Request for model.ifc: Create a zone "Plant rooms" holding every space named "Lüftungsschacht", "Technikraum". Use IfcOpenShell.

First a look at what the model holds.

```python
import ifcopenshell

model = ifcopenshell.open("model.ifc")
print(model.schema)
seen = {}
for space in model.by_type("IfcSpace"):
    seen[space.LongName] = seen.get(space.LongName, 0) + 1
for name, count in sorted(seen.items(), key=str):
    print(count, "x", name)
print("zones:", [z.Name for z in model.by_type("IfcZone")][:20])
```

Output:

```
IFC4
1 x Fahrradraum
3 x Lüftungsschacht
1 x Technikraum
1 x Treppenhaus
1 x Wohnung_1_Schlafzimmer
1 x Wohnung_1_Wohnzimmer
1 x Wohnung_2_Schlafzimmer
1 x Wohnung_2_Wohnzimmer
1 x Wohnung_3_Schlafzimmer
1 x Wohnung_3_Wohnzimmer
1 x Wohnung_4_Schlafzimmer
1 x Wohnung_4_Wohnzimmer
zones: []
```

```python
import ifcopenshell
import ifcopenshell.api.group
import ifcopenshell.api.root

model = ifcopenshell.open("model.ifc")

names = {"Lüftungsschacht", "Technikraum"}
spaces = [s for s in model.by_type("IfcSpace") if s.LongName in names]

zone = ifcopenshell.api.root.create_entity(model, ifc_class="IfcZone", name="Plant rooms")
ifcopenshell.api.group.assign_group(model, products=spaces, group=zone)
print(len(spaces), "spaces in", zone.Name)

model.write("model_v2.ifc")
```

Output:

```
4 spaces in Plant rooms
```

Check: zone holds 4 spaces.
